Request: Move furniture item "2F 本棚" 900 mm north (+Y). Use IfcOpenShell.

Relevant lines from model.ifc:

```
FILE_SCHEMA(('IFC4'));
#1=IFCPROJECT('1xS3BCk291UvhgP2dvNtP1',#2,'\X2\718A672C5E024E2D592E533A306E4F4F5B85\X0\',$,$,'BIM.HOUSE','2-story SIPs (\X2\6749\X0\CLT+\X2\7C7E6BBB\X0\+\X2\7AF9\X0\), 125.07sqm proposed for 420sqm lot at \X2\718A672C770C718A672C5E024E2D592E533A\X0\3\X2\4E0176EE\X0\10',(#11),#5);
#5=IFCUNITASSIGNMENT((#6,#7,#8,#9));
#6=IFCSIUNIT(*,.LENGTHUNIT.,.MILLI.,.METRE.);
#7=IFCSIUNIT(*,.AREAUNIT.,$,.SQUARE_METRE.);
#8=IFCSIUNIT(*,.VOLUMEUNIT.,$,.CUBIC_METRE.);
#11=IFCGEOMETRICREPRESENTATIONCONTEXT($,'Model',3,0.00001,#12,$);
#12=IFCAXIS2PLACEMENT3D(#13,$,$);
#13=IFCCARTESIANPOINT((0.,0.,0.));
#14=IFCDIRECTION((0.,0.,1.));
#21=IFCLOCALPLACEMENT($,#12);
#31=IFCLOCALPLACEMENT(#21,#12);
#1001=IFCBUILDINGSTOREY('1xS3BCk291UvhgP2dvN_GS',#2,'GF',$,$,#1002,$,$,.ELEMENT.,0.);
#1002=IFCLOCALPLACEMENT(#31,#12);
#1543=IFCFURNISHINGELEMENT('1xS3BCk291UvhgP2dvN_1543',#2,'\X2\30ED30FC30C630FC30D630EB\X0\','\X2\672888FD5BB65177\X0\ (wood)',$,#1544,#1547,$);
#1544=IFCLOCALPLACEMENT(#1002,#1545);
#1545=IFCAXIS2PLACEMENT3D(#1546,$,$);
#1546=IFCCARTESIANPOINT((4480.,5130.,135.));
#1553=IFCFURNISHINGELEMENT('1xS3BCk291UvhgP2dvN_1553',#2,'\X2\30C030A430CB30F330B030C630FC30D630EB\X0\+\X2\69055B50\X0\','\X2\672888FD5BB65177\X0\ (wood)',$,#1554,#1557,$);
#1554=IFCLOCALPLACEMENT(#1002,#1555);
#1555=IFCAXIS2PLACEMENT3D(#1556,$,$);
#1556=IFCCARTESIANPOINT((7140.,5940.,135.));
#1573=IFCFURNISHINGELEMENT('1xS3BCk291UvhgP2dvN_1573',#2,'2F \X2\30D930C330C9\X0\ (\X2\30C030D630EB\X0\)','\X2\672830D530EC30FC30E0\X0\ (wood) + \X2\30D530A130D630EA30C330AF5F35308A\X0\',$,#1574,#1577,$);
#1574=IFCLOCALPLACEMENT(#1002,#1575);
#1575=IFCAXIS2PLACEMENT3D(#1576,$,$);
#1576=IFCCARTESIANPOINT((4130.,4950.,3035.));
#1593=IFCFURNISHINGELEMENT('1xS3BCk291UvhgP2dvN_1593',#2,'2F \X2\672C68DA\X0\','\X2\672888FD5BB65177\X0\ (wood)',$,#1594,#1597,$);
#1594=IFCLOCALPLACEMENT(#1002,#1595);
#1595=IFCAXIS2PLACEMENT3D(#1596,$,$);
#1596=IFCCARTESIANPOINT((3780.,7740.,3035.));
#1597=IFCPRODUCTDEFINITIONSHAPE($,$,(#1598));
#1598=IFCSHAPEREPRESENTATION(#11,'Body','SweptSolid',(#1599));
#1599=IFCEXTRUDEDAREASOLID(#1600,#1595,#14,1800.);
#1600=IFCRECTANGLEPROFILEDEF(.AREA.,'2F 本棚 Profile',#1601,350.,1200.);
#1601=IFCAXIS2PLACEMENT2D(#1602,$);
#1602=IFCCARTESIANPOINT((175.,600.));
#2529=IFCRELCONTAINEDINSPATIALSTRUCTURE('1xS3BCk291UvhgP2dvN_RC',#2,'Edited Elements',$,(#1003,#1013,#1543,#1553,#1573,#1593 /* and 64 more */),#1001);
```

```python
import ifcopenshell
import ifcopenshell.api.geometry
import ifcopenshell.util.placement

model = ifcopenshell.open("model.ifc")

item = model.by_guid("1xS3BCk291UvhgP2dvN_1593")
matrix = ifcopenshell.util.placement.get_local_placement(item.ObjectPlacement)
matrix[1, 3] += 900.0
ifcopenshell.api.geometry.edit_object_placement(model, product=item, matrix=matrix, is_si=False)

print(ifcopenshell.util.placement.get_local_placement(item.ObjectPlacement).round(3) + 0.0)

model.write("model-out.ifc")
```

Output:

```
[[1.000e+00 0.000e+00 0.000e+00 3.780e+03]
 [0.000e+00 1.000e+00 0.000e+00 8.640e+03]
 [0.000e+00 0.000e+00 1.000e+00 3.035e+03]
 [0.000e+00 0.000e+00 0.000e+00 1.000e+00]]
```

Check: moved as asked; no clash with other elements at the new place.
